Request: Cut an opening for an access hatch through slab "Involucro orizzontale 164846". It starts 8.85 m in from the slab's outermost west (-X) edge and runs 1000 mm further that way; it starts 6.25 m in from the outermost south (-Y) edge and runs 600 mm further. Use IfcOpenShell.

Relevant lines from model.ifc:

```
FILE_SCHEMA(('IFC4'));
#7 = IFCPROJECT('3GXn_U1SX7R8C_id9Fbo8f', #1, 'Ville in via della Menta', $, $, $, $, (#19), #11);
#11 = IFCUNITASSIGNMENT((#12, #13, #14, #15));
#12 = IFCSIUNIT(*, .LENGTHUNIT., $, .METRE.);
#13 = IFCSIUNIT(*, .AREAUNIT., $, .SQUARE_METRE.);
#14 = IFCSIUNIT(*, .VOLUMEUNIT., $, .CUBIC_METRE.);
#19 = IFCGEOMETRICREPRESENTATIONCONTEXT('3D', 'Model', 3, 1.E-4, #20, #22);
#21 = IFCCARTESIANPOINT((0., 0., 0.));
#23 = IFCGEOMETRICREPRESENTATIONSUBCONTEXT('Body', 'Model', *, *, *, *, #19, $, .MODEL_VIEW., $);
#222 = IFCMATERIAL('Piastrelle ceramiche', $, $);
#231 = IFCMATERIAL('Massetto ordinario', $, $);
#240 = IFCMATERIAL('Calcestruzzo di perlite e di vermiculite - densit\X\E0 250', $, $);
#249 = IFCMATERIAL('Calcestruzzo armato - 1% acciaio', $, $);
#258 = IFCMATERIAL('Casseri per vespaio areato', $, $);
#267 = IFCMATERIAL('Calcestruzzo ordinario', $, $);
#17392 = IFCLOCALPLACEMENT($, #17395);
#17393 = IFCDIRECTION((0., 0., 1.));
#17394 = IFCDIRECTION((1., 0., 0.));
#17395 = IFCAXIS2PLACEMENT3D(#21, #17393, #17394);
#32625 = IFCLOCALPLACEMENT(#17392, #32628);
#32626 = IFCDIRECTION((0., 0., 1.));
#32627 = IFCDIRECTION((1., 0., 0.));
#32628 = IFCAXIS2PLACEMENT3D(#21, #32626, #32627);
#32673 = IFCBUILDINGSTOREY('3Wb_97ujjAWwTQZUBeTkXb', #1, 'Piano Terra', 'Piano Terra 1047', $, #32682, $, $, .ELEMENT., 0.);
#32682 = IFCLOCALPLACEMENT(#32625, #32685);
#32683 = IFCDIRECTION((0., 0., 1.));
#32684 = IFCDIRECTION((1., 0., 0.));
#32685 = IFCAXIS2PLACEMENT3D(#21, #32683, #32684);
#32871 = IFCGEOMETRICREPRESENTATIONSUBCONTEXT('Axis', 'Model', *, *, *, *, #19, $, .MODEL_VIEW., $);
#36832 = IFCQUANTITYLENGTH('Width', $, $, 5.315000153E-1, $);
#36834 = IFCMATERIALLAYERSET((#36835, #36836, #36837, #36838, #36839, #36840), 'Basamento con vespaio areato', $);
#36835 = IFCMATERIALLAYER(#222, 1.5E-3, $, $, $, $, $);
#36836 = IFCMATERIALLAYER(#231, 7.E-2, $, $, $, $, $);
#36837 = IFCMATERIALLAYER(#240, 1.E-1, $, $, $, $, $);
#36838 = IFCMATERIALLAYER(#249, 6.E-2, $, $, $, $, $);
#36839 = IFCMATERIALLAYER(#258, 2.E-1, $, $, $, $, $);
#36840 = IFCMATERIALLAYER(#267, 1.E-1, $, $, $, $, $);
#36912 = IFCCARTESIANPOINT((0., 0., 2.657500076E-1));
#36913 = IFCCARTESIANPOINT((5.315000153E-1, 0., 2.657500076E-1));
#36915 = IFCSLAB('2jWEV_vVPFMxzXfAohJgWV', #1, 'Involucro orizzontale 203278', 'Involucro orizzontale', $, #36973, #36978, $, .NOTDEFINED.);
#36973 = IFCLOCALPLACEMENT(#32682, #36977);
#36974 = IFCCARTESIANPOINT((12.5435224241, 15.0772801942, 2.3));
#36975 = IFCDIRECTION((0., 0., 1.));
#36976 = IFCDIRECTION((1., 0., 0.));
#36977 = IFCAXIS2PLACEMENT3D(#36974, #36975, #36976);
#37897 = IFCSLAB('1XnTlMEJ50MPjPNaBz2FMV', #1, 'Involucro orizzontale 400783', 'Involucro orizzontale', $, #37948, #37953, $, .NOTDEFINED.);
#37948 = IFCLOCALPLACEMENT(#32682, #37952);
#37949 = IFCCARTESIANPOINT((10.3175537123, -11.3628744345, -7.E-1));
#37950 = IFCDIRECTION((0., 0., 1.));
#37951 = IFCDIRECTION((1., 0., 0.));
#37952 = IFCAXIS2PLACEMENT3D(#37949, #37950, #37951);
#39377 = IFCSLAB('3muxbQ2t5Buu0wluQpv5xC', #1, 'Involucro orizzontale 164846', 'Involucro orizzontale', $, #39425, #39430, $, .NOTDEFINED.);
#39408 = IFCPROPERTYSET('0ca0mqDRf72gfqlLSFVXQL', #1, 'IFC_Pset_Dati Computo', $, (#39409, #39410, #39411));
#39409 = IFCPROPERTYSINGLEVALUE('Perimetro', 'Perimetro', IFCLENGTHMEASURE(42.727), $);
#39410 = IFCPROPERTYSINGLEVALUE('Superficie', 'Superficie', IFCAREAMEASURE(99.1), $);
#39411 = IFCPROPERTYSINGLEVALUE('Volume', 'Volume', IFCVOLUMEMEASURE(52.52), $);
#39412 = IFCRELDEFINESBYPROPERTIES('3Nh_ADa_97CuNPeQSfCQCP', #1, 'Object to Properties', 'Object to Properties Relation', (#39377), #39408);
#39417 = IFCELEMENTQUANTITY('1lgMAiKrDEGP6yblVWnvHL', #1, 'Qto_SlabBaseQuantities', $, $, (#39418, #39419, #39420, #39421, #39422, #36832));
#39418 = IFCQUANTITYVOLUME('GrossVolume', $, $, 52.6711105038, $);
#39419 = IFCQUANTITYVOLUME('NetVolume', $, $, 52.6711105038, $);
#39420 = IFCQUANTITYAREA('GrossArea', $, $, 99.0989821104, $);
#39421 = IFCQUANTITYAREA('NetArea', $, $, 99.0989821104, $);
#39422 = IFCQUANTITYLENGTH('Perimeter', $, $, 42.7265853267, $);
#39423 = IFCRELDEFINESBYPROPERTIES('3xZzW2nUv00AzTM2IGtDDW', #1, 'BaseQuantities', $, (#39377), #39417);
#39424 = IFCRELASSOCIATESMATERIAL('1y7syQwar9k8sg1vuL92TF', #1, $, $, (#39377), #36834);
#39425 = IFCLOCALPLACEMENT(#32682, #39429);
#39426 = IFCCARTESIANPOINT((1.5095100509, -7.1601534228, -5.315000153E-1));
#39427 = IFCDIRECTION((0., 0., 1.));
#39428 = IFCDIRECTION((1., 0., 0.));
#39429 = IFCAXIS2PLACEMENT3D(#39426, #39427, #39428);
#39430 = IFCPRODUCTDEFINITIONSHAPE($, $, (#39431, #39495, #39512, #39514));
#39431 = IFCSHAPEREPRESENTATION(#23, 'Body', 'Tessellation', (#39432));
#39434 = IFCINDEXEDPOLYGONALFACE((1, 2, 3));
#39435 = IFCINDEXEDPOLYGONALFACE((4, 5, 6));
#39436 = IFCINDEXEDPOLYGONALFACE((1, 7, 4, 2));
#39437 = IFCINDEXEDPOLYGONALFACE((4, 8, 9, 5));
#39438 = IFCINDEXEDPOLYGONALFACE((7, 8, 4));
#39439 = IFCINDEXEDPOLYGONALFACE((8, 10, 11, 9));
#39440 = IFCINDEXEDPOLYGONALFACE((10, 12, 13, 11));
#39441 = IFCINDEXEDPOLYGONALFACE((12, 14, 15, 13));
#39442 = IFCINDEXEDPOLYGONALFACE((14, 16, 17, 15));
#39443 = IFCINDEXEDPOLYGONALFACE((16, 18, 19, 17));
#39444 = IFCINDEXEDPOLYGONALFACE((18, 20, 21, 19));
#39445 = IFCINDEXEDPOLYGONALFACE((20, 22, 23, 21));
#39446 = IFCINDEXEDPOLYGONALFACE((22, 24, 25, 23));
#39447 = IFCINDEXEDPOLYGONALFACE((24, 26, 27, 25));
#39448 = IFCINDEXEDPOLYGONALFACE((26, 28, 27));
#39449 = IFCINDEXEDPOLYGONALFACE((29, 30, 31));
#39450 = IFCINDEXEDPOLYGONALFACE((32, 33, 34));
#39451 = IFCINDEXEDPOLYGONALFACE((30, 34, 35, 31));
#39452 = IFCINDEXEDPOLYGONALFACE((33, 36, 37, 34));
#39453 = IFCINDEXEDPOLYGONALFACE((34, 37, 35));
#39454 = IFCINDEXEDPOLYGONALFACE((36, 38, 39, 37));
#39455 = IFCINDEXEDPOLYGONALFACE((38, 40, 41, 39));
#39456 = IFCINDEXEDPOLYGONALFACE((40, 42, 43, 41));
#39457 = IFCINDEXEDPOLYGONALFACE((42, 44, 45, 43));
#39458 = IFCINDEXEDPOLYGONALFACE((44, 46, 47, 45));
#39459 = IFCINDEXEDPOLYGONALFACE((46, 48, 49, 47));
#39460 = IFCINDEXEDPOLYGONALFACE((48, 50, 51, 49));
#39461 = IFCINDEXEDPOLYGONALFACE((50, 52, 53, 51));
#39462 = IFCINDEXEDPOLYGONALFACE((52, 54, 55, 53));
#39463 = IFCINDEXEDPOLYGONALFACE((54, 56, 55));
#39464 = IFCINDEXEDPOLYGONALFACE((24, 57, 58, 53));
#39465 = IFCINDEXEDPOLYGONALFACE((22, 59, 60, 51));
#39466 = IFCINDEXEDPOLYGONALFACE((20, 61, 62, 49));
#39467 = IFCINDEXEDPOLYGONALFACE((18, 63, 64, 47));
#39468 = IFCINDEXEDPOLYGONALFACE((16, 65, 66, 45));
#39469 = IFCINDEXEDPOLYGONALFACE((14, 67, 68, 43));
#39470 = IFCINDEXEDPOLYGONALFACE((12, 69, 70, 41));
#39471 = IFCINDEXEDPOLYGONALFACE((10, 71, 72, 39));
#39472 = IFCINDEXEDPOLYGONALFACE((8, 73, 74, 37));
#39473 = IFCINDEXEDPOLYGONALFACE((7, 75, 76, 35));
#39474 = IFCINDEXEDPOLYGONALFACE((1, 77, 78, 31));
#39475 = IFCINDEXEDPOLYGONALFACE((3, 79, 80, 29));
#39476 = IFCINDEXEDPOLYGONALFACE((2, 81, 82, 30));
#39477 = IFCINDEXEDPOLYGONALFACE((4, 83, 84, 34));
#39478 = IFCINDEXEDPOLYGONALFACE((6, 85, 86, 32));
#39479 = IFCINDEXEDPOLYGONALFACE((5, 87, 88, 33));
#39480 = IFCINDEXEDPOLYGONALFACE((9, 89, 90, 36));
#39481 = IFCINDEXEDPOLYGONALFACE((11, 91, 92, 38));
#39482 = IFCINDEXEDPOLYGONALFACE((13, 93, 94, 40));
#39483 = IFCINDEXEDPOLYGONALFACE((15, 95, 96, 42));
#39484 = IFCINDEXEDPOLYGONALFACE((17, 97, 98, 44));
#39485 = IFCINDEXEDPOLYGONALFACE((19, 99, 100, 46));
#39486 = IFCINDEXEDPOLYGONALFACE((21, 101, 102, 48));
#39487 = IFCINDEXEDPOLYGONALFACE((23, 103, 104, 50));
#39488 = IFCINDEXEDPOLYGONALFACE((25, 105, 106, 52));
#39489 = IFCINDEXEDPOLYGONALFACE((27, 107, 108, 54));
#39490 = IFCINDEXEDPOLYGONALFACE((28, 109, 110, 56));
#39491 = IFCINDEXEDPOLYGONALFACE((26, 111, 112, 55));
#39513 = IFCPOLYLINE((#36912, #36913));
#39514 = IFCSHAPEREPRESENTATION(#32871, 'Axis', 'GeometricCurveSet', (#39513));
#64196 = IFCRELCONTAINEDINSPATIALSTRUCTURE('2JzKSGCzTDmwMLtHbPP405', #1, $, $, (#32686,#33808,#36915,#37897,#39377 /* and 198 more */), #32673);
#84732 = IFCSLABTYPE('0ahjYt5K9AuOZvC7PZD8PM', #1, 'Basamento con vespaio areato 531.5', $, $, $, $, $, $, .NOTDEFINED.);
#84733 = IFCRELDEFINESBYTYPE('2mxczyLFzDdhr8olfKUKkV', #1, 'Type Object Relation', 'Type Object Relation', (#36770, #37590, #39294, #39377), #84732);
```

```python
import numpy as np
import ifcopenshell
import ifcopenshell.api.feature
import ifcopenshell.api.geometry
import ifcopenshell.api.pset
import ifcopenshell.api.root
import ifcopenshell.geom
import ifcopenshell.util.element
import ifcopenshell.util.placement
import ifcopenshell.util.representation
import ifcopenshell.util.shape
import ifcopenshell.util.unit

model = ifcopenshell.open("model.ifc")
unit_scale = ifcopenshell.util.unit.calculate_unit_scale(model)
area_scale = ifcopenshell.util.unit.calculate_unit_scale(model, "AREAUNIT")
volume_scale = ifcopenshell.util.unit.calculate_unit_scale(model, "VOLUMEUNIT")
settings = ifcopenshell.geom.settings()


def volume(element):
    """Net volume in cubic metres, openings subtracted."""
    shape = ifcopenshell.geom.create_shape(settings, element)
    return ifcopenshell.util.shape.get_volume(shape.geometry)


slab = model.by_guid("3muxbQ2t5Buu0wluQpv5xC")
before = volume(slab)

# Extent in the slab's own axes, in metres. The edges named are its -X and -Y sides.
slab_shape = ifcopenshell.geom.create_shape(settings, slab)
vertices = ifcopenshell.util.shape.get_vertices(slab_shape.geometry)
x_min, y_min, bottom = vertices.min(axis=0)
top = vertices[:, 2].max()

opening = ifcopenshell.api.root.create_entity(model, ifc_class="IfcOpeningElement", name="Access hatch opening", predefined_type="OPENING")
context = ifcopenshell.util.representation.get_context(model, "Model", "Body", "MODEL_VIEW")
width, depth = 1, 0.6
outline = [(0.0, 0.0), (width, 0.0), (width, depth), (0.0, depth), (0.0, 0.0)]
# Overshoot both faces by 50 mm so the cut is clean.
shape = ifcopenshell.api.geometry.add_slab_representation(
    model, context=context, depth=top - bottom + 0.1, polyline=outline
)
ifcopenshell.api.geometry.assign_representation(model, product=opening, representation=shape)

matrix = ifcopenshell.util.placement.get_local_placement(slab.ObjectPlacement)
matrix[:, 3] = matrix @ np.append(np.array([x_min + 8.85, y_min + 6.25, bottom - 0.05]) / unit_scale, 1.0)
ifcopenshell.api.geometry.edit_object_placement(model, product=opening, matrix=matrix, is_si=False)
ifcopenshell.api.feature.add_feature(model, feature=opening, element=slab)

after = volume(slab)

# Update the slab's stored quantities.
pset = model.by_id(ifcopenshell.util.element.get_pset(slab, "IFC_Pset_Dati Computo", should_inherit=False)["id"])
ifcopenshell.api.pset.edit_pset(model, pset=pset, properties={
    "Superficie": model.create_entity("IfcAreaMeasure", after / (top - bottom) / area_scale),
    "Volume": model.create_entity("IfcVolumeMeasure", after / volume_scale),
})
qto = model.by_id(ifcopenshell.util.element.get_pset(slab, "Qto_SlabBaseQuantities", should_inherit=False)["id"])
ifcopenshell.api.pset.edit_qto(model, qto=qto, properties={
    "NetVolume": after / volume_scale,
    "NetArea": after / (top - bottom) / area_scale,
})

print(f"slab volume {before:.3f} -> {after:.3f} m3")

model.write("model-out.ifc")
```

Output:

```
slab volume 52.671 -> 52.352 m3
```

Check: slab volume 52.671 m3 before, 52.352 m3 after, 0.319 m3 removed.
